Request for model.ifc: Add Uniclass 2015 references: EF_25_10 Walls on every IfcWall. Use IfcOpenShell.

First a look at what the model holds.

```python
import ifcopenshell

model = ifcopenshell.open("model.ifc")
print(model.schema)
print("classifications:", [c.Name for c in model.by_type("IfcClassification")])
for ifc_class in ("IfcDoor", "IfcRoof", "IfcStair", "IfcWall", "IfcWindow"):
    print(ifc_class, len(model.by_type(ifc_class)))
```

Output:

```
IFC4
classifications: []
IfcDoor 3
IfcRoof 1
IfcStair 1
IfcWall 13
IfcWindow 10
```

```python
import ifcopenshell
import ifcopenshell.api.classification

model = ifcopenshell.open("model.ifc")

system = ifcopenshell.api.classification.add_classification(model, classification="Uniclass 2015")

codes = {
    "IfcWall": ("EF_25_10", "Walls"),
}
for ifc_class, (code, name) in codes.items():
    products = model.by_type(ifc_class)
    ifcopenshell.api.classification.add_reference(
        model, products=products, classification=system, identification=code, name=name
    )
    print(code, len(products))

model.write("model_v2.ifc")
```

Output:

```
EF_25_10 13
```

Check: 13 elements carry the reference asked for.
